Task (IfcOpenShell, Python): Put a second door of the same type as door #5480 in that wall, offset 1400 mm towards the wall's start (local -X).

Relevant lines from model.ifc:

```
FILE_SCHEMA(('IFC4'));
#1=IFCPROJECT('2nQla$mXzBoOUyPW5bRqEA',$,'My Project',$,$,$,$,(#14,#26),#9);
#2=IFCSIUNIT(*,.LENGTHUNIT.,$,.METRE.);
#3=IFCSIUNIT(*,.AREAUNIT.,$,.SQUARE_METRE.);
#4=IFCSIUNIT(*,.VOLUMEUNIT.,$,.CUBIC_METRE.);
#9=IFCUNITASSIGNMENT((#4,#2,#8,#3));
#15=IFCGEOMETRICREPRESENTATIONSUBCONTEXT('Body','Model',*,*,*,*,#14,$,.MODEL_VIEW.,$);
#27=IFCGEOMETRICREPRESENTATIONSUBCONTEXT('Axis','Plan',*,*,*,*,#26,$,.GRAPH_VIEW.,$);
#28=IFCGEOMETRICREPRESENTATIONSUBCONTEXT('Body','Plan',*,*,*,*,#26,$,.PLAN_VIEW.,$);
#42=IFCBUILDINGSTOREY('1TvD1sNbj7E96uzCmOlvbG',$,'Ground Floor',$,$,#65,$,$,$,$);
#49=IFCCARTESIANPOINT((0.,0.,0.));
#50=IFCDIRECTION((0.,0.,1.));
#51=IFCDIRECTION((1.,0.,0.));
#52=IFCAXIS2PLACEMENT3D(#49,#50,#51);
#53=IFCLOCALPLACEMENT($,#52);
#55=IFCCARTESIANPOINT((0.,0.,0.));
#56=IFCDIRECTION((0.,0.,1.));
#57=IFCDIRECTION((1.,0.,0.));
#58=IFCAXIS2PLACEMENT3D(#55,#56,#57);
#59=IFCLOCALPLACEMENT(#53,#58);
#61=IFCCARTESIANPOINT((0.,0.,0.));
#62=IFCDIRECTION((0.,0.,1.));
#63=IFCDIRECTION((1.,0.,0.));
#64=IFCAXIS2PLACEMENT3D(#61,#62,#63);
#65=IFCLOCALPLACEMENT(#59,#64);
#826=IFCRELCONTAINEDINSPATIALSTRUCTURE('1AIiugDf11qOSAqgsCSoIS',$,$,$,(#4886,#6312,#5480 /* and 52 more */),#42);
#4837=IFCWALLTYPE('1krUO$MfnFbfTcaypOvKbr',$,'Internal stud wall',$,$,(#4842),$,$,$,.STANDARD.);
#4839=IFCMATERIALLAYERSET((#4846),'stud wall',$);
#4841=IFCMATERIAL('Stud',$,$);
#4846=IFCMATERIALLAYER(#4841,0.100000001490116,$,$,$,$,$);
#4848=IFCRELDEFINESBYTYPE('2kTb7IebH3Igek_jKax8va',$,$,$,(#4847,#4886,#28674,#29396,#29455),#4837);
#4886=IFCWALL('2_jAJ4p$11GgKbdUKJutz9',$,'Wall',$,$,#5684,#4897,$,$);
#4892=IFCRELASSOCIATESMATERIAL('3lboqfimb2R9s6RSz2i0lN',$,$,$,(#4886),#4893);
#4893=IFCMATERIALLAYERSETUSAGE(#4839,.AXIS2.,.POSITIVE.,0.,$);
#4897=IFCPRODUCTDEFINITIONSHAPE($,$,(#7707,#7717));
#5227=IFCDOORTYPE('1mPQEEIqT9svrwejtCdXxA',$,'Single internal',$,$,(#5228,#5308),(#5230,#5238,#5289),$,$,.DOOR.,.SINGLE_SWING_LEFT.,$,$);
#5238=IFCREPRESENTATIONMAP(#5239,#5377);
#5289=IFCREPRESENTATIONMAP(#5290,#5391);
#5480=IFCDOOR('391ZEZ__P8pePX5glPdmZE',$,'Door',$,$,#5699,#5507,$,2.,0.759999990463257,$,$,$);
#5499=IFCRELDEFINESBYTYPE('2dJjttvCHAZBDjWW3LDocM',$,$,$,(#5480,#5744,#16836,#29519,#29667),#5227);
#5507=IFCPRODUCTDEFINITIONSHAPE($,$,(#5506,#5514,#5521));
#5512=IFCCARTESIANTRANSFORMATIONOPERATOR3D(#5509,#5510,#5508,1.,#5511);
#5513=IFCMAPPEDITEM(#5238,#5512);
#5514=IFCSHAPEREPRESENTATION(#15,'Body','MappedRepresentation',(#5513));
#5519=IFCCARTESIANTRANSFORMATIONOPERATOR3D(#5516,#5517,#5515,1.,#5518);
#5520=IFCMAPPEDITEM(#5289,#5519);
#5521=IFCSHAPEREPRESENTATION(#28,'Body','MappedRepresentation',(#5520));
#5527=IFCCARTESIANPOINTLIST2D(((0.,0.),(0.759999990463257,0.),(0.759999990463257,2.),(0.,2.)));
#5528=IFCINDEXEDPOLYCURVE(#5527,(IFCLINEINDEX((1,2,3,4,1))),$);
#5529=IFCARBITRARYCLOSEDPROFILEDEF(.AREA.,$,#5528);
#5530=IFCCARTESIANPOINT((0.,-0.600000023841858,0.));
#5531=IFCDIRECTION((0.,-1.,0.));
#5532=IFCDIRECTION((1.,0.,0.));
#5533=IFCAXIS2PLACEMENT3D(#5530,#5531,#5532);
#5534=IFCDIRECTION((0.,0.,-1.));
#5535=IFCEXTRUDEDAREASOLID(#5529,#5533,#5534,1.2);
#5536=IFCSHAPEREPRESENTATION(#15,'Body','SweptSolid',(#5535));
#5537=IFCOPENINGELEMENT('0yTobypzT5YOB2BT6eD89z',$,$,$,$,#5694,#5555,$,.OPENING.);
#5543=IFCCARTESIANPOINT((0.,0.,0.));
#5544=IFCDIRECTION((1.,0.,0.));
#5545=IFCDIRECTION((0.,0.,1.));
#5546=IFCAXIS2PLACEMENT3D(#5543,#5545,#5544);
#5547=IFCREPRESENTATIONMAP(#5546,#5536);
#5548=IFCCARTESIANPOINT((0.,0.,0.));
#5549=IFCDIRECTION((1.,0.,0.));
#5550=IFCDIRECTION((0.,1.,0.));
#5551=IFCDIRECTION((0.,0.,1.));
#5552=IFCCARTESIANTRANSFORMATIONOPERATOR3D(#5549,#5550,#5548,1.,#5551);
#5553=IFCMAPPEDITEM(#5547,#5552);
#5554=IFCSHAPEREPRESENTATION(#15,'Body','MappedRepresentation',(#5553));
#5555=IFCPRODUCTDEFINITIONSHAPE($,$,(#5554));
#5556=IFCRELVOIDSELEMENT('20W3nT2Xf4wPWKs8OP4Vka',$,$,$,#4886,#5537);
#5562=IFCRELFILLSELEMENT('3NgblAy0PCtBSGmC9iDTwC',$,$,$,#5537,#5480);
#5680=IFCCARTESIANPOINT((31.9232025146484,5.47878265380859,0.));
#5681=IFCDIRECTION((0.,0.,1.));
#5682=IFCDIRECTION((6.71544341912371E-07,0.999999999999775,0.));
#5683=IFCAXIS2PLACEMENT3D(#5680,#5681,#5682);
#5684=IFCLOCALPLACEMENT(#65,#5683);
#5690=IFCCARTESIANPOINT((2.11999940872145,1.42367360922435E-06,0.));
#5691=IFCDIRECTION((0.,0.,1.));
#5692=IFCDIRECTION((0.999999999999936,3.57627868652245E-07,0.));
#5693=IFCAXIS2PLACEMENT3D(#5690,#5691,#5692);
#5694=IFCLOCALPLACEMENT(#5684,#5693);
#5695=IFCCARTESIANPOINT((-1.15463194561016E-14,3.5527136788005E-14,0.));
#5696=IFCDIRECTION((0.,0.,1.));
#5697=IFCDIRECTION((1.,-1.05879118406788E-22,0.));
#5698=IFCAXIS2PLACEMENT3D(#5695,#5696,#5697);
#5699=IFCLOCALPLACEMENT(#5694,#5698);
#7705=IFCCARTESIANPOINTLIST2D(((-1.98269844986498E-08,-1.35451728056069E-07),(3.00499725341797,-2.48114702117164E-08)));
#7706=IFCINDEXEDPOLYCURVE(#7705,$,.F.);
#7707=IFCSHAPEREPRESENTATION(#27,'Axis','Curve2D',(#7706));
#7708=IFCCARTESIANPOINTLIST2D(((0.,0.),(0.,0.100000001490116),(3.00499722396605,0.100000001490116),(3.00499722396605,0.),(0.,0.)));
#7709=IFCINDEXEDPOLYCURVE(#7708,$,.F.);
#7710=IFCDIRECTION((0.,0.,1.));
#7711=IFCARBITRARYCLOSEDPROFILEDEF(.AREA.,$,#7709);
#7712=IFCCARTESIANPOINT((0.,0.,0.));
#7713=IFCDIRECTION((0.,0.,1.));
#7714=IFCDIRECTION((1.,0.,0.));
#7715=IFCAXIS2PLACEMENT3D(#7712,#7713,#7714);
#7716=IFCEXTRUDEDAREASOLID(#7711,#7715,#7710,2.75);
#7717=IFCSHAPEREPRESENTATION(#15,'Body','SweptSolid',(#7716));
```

```python
import ifcopenshell
import ifcopenshell.api.feature
import ifcopenshell.api.geometry
import ifcopenshell.api.root
import ifcopenshell.geom
import ifcopenshell.util.element
import ifcopenshell.util.placement
import ifcopenshell.util.shape

model = ifcopenshell.open("model.ifc")
settings = ifcopenshell.geom.settings()


def volume(element):
    """Net volume in cubic metres, openings subtracted."""
    shape = ifcopenshell.geom.create_shape(settings, element)
    return ifcopenshell.util.shape.get_volume(shape.geometry)


door = model.by_guid("391ZEZ__P8pePX5glPdmZE")
opening = door.FillsVoids[0].RelatingOpeningElement
wall = opening.VoidsElements[0].RelatingBuildingElement
before = volume(wall)
shift = ifcopenshell.util.placement.get_local_placement(wall.ObjectPlacement)[:3, 0] * -1.4

# copy_class copies the void relationship, type, container and properties, but no geometry.
new_opening = ifcopenshell.api.root.copy_class(model, product=opening)
new_opening.Representation = ifcopenshell.util.element.copy_deep(
    model, opening.Representation, exclude=["IfcGeometricRepresentationContext", "IfcRepresentationMap"]
)
new_door = ifcopenshell.api.root.copy_class(model, product=door)
new_door.Representation = ifcopenshell.util.element.copy_deep(
    model, door.Representation, exclude=["IfcGeometricRepresentationContext", "IfcRepresentationMap"]
)
ifcopenshell.api.feature.add_filling(model, opening=new_opening, element=new_door)

for old, new in ((opening, new_opening), (door, new_door)):
    matrix = ifcopenshell.util.placement.get_local_placement(old.ObjectPlacement)
    matrix[:3, 3] += shift
    ifcopenshell.api.geometry.edit_object_placement(model, product=new, matrix=matrix, is_si=False)

after = volume(wall)

print(f"wall volume {before:.3f} -> {after:.3f} m3")

model.write("model_updated.ifc")
```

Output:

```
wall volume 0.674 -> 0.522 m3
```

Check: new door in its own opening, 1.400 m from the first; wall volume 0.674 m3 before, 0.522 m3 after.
